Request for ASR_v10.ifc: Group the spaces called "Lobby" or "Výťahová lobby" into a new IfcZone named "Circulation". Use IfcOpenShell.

First a look at what the model holds.

```python
import ifcopenshell

model = ifcopenshell.open("ASR_v10.ifc")
print(model.schema)
seen = {}
for space in model.by_type("IfcSpace"):
    seen[space.LongName] = seen.get(space.LongName, 0) + 1
for name, count in sorted(seen.items(), key=str):
    print(count, "x", name)
print("zones:", [z.Name for z in model.by_type("IfcZone")][:20])
```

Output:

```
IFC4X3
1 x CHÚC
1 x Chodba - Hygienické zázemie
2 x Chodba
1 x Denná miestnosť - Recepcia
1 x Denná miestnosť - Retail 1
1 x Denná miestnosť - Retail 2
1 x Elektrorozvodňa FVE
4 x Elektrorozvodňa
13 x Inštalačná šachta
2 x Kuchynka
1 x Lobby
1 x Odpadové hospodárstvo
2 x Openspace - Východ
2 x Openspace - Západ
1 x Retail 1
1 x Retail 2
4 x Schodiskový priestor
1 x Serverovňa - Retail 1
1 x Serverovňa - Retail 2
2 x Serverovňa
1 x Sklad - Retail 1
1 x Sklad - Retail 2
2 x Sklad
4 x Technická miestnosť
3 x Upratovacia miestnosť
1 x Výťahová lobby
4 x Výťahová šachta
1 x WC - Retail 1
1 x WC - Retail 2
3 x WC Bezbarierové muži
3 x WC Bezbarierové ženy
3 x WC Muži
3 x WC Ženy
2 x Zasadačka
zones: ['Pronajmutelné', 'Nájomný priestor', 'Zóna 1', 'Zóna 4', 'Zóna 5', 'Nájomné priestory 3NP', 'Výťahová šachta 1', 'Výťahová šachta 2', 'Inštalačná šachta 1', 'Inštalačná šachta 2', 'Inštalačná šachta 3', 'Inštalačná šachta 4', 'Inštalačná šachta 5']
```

```python
import ifcopenshell
import ifcopenshell.api.group
import ifcopenshell.api.root

model = ifcopenshell.open("ASR_v10.ifc")

names = {"Lobby", "Výťahová lobby"}
spaces = [s for s in model.by_type("IfcSpace") if s.LongName in names]

zone = ifcopenshell.api.root.create_entity(model, ifc_class="IfcZone", name="Circulation")
ifcopenshell.api.group.assign_group(model, products=spaces, group=zone)
print(len(spaces), "spaces in", zone.Name)

model.write("ASR_v10-out.ifc")
```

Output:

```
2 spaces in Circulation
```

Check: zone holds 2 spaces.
